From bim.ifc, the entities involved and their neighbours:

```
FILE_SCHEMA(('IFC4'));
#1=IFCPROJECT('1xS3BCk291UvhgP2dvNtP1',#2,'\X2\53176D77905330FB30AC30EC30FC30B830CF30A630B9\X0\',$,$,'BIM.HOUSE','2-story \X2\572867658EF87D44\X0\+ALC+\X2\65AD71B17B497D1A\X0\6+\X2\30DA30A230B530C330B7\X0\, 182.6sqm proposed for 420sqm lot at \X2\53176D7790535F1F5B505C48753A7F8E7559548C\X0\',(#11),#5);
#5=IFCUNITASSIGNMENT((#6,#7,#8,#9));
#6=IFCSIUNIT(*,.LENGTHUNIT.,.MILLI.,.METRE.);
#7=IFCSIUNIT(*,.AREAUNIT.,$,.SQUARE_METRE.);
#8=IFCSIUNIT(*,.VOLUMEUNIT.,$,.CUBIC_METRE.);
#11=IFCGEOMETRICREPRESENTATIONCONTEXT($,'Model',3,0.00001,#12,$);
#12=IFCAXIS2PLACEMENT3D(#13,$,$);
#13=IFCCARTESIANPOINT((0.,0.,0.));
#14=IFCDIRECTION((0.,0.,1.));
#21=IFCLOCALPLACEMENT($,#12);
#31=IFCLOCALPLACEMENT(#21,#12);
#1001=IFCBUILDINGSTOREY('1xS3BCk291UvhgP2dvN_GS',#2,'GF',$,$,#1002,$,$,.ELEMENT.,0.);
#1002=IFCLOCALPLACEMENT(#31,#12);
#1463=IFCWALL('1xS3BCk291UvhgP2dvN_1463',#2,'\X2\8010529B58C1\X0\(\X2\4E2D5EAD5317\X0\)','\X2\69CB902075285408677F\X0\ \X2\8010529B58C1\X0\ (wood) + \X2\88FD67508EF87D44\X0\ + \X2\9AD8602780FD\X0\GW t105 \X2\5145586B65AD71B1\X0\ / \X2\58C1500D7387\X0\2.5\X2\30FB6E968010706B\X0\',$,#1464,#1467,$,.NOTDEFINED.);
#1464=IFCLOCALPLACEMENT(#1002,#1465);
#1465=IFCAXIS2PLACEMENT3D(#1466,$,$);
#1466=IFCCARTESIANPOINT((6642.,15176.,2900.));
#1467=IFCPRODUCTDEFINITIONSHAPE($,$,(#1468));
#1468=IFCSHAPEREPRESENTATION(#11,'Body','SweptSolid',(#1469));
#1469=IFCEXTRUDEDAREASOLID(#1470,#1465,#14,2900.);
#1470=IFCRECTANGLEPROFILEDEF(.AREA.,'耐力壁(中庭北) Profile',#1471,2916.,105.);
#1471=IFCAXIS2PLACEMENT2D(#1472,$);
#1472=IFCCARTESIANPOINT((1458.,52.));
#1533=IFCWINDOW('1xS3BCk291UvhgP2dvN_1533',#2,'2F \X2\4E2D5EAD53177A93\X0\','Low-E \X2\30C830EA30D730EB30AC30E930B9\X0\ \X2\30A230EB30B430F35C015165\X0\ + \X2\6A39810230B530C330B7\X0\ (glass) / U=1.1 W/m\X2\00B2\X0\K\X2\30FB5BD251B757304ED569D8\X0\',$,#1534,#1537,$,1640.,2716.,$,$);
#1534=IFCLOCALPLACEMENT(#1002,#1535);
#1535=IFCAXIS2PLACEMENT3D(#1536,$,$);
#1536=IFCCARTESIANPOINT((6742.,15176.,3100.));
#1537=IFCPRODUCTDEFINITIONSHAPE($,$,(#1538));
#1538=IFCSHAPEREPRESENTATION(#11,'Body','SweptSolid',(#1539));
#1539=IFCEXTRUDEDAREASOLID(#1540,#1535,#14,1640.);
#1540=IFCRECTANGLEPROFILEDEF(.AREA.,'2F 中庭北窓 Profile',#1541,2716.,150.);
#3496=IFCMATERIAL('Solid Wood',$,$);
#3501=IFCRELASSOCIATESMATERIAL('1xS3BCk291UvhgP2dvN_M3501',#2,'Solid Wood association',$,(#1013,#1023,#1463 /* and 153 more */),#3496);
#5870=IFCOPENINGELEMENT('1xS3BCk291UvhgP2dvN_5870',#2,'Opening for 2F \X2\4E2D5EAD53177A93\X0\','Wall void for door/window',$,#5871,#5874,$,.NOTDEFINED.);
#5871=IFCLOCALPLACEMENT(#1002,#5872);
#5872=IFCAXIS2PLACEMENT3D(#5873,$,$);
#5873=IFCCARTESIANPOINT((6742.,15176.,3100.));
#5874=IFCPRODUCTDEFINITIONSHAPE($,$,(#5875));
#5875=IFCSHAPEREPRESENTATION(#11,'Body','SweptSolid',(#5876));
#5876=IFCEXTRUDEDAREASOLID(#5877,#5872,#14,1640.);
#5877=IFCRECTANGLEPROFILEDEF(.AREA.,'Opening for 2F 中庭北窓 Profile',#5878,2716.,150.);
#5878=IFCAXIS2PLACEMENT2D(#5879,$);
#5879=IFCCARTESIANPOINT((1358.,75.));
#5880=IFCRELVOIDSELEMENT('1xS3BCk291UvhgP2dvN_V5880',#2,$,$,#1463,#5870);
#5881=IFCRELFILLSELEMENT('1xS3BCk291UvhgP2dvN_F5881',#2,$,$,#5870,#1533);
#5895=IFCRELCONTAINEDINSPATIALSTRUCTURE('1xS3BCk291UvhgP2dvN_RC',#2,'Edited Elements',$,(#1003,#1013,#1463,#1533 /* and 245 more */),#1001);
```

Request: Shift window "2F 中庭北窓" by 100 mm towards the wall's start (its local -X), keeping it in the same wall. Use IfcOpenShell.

```python
import ifcopenshell
import ifcopenshell.api.geometry
import ifcopenshell.util.placement

model = ifcopenshell.open("bim.ifc")

window = model.by_guid("1xS3BCk291UvhgP2dvN_1533")
opening = window.FillsVoids[0].RelatingOpeningElement
wall = opening.VoidsElements[0].RelatingBuildingElement

wall_matrix = ifcopenshell.util.placement.get_local_placement(wall.ObjectPlacement)
shift = wall_matrix[:3, 0] * -100.0
before = ifcopenshell.util.placement.get_local_placement(window.ObjectPlacement)[:3, 3].copy()

# The window is not placed relative to its opening, so move both.
for product in (opening, window):
    matrix = ifcopenshell.util.placement.get_local_placement(product.ObjectPlacement)
    matrix[:3, 3] += shift
    ifcopenshell.api.geometry.edit_object_placement(model, product=product, matrix=matrix, is_si=False)

after = ifcopenshell.util.placement.get_local_placement(window.ObjectPlacement)[:3, 3]
print("window moved by", (after - before).round(3) + 0.0)

model.write("bim-out.ifc")
```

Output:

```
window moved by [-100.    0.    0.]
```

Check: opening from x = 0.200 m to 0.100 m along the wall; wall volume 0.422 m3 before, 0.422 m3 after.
